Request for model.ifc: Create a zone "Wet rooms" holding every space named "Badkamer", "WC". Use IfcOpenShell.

First a look at what the model holds.

```python
import ifcopenshell

model = ifcopenshell.open("model.ifc")
print(model.schema)
seen = {}
for space in model.by_type("IfcSpace"):
    seen[space.LongName] = seen.get(space.LongName, 0) + 1
for name, count in sorted(seen.items(), key=str):
    print(count, "x", name)
print("zones:", [z.Name for z in model.by_type("IfcZone")][:20])
```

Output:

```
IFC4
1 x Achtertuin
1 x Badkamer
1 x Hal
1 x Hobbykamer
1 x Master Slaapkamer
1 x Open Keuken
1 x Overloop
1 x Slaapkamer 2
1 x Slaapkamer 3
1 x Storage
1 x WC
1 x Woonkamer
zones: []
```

```python
import ifcopenshell
import ifcopenshell.api.group
import ifcopenshell.api.root

model = ifcopenshell.open("model.ifc")

names = {"Badkamer", "WC"}
spaces = [s for s in model.by_type("IfcSpace") if s.LongName in names]

zone = ifcopenshell.api.root.create_entity(model, ifc_class="IfcZone", name="Wet rooms")
ifcopenshell.api.group.assign_group(model, products=spaces, group=zone)
print(len(spaces), "spaces in", zone.Name)

model.write("model_updated.ifc")
```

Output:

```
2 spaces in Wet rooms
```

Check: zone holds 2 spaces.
